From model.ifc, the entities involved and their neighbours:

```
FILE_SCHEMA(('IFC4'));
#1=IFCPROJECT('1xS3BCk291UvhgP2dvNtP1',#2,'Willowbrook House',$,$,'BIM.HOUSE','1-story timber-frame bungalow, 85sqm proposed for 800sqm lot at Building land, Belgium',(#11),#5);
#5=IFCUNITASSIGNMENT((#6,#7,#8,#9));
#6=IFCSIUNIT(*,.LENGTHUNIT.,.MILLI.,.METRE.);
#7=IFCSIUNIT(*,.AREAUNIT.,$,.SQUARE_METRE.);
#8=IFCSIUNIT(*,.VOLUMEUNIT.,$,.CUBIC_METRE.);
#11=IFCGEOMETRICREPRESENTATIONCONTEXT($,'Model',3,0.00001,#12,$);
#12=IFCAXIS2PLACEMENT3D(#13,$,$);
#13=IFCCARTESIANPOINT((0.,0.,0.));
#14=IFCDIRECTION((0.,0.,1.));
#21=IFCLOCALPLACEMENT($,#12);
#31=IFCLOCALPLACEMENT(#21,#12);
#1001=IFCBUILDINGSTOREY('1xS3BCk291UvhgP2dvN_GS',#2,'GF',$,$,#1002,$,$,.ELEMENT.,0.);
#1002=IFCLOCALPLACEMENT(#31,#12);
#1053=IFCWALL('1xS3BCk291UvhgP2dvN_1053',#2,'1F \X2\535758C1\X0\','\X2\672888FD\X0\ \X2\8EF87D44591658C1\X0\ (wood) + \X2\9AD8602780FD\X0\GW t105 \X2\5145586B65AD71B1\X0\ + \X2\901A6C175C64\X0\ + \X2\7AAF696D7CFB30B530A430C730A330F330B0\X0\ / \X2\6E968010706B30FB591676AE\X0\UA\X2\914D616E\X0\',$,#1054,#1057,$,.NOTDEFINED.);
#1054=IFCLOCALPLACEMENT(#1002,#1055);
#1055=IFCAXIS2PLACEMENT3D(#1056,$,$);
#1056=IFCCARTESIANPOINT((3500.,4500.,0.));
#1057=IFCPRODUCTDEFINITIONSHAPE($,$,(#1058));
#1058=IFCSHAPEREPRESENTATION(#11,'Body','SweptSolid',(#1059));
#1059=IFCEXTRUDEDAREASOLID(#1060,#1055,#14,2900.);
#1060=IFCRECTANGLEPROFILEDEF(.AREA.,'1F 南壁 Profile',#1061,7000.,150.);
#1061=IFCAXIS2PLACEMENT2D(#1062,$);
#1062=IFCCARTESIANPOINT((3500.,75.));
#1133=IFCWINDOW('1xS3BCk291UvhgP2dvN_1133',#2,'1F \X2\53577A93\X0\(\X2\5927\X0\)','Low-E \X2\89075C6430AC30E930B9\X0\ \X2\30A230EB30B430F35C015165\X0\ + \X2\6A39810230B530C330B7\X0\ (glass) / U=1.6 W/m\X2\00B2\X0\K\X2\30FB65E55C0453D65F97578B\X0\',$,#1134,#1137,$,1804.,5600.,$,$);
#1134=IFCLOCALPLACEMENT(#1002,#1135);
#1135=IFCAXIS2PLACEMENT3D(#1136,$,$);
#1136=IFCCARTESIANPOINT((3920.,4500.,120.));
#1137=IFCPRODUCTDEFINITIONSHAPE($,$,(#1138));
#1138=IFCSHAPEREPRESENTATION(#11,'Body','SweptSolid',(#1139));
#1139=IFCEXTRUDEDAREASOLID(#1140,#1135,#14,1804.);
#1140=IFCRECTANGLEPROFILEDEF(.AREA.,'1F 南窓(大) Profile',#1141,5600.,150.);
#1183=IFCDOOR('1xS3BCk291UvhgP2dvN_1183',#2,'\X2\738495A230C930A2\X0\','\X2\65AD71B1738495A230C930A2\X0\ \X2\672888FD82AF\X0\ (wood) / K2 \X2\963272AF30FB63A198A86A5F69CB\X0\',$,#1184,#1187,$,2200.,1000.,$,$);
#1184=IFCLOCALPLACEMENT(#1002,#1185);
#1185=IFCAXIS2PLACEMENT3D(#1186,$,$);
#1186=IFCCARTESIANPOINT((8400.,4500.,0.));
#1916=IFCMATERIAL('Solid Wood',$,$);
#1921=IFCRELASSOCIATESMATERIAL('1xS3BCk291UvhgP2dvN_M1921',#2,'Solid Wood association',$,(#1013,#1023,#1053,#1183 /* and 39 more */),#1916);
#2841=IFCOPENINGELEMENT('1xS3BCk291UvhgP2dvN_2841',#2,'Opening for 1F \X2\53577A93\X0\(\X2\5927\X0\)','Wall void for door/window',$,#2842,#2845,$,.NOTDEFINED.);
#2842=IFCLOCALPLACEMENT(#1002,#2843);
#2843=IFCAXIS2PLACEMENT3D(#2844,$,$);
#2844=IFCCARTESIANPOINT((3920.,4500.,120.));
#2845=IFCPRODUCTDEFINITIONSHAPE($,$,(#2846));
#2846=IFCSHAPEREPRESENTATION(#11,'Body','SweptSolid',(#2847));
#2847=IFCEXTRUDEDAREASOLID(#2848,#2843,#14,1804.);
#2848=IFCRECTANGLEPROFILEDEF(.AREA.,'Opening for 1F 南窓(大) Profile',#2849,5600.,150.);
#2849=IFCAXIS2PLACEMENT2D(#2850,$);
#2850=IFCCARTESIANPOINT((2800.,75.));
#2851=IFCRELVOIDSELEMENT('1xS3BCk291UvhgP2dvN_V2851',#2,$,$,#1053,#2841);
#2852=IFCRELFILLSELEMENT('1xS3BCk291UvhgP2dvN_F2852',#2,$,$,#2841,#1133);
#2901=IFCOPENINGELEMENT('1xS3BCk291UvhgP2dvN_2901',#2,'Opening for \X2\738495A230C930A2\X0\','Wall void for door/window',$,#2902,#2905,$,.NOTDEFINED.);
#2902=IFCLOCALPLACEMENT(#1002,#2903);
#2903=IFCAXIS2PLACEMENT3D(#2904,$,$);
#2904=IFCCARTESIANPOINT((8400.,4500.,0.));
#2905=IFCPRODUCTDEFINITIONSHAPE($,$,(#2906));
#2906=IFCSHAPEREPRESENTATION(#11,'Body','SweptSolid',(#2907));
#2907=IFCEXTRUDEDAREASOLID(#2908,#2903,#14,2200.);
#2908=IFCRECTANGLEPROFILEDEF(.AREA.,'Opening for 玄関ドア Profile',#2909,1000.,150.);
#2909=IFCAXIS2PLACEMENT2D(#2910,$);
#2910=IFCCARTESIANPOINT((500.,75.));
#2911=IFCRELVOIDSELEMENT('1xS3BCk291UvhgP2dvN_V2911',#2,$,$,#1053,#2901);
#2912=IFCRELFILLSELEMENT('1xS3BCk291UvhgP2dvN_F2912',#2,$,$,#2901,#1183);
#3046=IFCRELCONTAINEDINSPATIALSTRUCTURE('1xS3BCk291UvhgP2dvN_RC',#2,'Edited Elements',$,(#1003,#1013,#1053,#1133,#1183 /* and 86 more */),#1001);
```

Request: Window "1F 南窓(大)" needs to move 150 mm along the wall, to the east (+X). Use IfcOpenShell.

```python
import ifcopenshell
import ifcopenshell.api.geometry
import ifcopenshell.util.placement
import ifcopenshell.util.unit

model = ifcopenshell.open("model.ifc")
unit_scale = ifcopenshell.util.unit.calculate_unit_scale(model)

window = model.by_guid("1xS3BCk291UvhgP2dvN_1133")
opening = window.FillsVoids[0].RelatingOpeningElement
wall = opening.VoidsElements[0].RelatingBuildingElement

wall_matrix = ifcopenshell.util.placement.get_local_placement(wall.ObjectPlacement)
shift = wall_matrix[:3, 0] * 0.15 / unit_scale
before = ifcopenshell.util.placement.get_local_placement(window.ObjectPlacement)[:3, 3].copy()

# The window is not placed relative to its opening, so move both.
for product in (opening, window):
    matrix = ifcopenshell.util.placement.get_local_placement(product.ObjectPlacement)
    matrix[:3, 3] += shift
    ifcopenshell.api.geometry.edit_object_placement(model, product=product, matrix=matrix, is_si=False)

after = ifcopenshell.util.placement.get_local_placement(window.ObjectPlacement)[:3, 3]
print("window moved by", (after - before).round(3) + 0.0)

model.write("model_updated.ifc")
```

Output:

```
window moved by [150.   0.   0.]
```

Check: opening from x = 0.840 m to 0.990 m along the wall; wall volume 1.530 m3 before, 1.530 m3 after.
